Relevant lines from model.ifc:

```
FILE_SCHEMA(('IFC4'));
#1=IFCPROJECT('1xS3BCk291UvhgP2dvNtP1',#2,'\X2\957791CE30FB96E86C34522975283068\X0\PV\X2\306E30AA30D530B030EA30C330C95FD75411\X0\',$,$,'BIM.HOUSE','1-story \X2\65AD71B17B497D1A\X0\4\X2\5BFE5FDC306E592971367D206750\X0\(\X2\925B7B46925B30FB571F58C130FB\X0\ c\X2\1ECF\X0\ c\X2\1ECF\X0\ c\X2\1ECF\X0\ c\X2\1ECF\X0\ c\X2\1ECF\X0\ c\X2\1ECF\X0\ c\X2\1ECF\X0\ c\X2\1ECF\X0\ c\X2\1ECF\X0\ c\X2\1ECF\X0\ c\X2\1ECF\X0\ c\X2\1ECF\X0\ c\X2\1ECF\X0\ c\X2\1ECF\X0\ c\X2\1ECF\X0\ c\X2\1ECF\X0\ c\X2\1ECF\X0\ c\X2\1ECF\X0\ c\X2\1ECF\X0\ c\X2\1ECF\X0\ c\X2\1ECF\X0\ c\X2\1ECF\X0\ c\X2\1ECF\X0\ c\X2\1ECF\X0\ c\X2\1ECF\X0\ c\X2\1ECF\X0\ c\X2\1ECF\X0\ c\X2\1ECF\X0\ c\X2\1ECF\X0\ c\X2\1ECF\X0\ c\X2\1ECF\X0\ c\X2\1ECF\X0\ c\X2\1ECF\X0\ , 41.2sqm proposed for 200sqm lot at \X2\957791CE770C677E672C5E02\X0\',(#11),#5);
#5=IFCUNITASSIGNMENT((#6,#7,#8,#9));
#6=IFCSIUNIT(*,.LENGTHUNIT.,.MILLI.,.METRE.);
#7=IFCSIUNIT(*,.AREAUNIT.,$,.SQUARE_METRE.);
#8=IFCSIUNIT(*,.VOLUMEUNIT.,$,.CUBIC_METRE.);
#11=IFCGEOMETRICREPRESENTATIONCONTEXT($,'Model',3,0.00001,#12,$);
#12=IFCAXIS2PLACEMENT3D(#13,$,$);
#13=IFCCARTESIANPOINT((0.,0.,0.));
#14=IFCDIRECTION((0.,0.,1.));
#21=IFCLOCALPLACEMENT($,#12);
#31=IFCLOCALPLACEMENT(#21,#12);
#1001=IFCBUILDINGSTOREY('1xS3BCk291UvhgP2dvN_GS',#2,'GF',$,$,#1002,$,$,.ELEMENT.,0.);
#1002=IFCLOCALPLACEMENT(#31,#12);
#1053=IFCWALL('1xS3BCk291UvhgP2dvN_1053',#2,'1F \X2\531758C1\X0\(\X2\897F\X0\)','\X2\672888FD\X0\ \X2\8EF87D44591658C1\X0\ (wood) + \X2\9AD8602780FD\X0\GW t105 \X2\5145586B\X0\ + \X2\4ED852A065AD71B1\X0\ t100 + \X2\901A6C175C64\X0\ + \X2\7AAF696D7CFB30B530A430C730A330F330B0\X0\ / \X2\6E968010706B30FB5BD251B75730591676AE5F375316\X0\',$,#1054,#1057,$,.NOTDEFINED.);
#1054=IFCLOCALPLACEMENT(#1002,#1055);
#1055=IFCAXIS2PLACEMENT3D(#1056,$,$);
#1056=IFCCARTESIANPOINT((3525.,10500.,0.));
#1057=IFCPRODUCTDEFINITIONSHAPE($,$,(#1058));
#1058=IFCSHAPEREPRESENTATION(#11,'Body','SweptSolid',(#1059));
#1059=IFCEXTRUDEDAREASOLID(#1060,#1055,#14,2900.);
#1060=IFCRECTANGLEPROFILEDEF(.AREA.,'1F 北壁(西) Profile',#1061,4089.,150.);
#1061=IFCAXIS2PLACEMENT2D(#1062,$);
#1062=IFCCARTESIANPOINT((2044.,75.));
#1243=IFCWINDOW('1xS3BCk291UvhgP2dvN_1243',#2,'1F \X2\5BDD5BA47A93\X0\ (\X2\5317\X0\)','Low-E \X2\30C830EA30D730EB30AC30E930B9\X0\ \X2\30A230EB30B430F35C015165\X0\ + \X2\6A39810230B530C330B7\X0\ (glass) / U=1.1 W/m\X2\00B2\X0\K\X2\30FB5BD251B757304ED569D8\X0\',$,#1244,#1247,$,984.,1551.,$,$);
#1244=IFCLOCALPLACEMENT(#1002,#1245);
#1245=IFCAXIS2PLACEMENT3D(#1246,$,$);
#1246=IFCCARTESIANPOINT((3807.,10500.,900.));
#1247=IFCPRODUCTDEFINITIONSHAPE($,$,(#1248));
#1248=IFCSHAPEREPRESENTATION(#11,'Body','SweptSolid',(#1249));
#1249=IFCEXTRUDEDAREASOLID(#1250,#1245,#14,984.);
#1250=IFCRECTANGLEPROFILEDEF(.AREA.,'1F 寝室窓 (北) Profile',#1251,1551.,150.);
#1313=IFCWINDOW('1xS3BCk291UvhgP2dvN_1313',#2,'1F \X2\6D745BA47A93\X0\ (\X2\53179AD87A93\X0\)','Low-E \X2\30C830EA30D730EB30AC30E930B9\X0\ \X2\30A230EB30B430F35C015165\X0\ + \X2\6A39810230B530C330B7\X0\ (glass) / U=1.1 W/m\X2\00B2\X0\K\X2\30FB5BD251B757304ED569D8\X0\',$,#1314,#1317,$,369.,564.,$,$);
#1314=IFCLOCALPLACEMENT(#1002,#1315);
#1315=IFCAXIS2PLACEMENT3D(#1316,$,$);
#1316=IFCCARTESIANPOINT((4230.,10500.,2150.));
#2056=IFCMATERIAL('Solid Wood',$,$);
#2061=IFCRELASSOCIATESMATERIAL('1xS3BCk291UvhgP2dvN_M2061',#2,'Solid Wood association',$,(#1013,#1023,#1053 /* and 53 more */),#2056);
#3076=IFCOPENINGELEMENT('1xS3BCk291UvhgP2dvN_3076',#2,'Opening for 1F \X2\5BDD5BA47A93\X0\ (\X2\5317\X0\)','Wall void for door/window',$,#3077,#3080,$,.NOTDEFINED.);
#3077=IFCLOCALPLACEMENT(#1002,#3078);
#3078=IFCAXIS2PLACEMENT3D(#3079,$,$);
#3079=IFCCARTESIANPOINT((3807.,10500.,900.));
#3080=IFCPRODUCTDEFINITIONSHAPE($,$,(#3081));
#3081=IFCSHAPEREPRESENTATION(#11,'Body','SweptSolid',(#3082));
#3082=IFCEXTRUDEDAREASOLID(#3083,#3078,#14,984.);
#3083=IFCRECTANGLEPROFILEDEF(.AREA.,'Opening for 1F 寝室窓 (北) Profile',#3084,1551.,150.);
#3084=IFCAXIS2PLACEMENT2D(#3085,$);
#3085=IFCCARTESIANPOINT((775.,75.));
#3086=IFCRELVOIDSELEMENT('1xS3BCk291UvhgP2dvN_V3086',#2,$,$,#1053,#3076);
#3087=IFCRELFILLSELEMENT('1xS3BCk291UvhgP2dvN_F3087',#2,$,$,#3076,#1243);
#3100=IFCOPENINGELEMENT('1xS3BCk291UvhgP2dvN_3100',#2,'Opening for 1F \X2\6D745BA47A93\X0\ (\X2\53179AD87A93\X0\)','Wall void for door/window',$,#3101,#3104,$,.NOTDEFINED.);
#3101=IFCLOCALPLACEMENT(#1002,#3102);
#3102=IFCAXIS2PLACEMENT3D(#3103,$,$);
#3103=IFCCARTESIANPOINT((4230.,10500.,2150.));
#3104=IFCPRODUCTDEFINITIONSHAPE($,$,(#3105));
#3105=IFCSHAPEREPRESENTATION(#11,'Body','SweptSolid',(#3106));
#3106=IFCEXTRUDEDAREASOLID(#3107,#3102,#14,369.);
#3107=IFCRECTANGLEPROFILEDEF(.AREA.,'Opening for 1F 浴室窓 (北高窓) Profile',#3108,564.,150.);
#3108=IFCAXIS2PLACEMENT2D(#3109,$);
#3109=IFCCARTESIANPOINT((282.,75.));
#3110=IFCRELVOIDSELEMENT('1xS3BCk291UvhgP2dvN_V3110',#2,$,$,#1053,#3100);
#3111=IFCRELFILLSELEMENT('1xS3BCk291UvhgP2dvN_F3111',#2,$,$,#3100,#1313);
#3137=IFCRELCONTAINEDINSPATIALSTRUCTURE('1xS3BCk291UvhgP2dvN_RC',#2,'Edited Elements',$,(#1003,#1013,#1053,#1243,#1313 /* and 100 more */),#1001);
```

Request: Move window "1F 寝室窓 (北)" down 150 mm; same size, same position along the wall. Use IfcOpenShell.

```python
import numpy as np
import ifcopenshell
import ifcopenshell.api.geometry
import ifcopenshell.util.placement
import ifcopenshell.util.unit

model = ifcopenshell.open("model.ifc")
unit_scale = ifcopenshell.util.unit.calculate_unit_scale(model)

window = model.by_guid("1xS3BCk291UvhgP2dvN_1243")
opening = window.FillsVoids[0].RelatingOpeningElement
dz = -0.15 / unit_scale

shift = np.array([0.0, 0.0, dz])
# The window is not placed relative to its opening, so move both.
for product in (opening, window):
    matrix = ifcopenshell.util.placement.get_local_placement(product.ObjectPlacement)
    matrix[:3, 3] += shift
    ifcopenshell.api.geometry.edit_object_placement(model, product=product, matrix=matrix, is_si=False)

print(f"moved by {dz * unit_scale:+.3f} m")

model.write("model_updated.ifc")
```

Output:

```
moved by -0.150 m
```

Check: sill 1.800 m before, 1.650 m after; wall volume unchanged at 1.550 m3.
